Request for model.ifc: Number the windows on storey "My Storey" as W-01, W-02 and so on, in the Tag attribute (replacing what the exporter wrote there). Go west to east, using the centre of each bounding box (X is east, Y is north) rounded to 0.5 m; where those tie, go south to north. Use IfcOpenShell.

First a look at what the model holds.

```python
import ifcopenshell
import ifcopenshell.util.element
import ifcopenshell.util.placement

model = ifcopenshell.open("model.ifc")
print(model.schema)
storey = next(s for s in model.by_type("IfcBuildingStorey") if s.Name == "My Storey")
windows = [e for e in ifcopenshell.util.element.get_decomposition(storey) if e.is_a("IfcWindow")]
for e in sorted(windows, key=lambda e: e.id()):
    origin = ifcopenshell.util.placement.get_local_placement(e.ObjectPlacement)[:3, 3]
    print(e.id(), e.Tag, e.Name, origin.round(2) + 0.0, sep=" | ")
```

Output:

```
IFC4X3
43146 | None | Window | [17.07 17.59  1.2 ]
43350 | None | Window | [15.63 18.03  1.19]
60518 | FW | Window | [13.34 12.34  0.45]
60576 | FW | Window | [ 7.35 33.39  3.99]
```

```python
import ifcopenshell
import ifcopenshell.geom
import ifcopenshell.util.element
import ifcopenshell.util.shape

model = ifcopenshell.open("model.ifc")
settings = ifcopenshell.geom.settings()
settings.set("use-world-coords", True)


def centre(element):
    shape = ifcopenshell.geom.create_shape(settings, element)
    return ifcopenshell.util.shape.get_bbox_centroid(shape.geometry)


storey = next(s for s in model.by_type("IfcBuildingStorey") if s.Name == "My Storey")
windows = [e for e in ifcopenshell.util.element.get_decomposition(storey) if e.is_a("IfcWindow")]

# Insertion points can sit at a corner or the storey origin, so sort by the geometry (in metres).
centres = {e: centre(e) for e in windows}
windows.sort(key=lambda e: (round(centres[e][0] / 0.5), centres[e][1]))

for i, e in enumerate(windows, start=1):
    number = f"W-{i:02d}"
    e.Tag = number
    print(e.id(), number)

model.write("model_edited.ifc")
```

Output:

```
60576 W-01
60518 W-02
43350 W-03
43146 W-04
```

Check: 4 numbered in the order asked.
